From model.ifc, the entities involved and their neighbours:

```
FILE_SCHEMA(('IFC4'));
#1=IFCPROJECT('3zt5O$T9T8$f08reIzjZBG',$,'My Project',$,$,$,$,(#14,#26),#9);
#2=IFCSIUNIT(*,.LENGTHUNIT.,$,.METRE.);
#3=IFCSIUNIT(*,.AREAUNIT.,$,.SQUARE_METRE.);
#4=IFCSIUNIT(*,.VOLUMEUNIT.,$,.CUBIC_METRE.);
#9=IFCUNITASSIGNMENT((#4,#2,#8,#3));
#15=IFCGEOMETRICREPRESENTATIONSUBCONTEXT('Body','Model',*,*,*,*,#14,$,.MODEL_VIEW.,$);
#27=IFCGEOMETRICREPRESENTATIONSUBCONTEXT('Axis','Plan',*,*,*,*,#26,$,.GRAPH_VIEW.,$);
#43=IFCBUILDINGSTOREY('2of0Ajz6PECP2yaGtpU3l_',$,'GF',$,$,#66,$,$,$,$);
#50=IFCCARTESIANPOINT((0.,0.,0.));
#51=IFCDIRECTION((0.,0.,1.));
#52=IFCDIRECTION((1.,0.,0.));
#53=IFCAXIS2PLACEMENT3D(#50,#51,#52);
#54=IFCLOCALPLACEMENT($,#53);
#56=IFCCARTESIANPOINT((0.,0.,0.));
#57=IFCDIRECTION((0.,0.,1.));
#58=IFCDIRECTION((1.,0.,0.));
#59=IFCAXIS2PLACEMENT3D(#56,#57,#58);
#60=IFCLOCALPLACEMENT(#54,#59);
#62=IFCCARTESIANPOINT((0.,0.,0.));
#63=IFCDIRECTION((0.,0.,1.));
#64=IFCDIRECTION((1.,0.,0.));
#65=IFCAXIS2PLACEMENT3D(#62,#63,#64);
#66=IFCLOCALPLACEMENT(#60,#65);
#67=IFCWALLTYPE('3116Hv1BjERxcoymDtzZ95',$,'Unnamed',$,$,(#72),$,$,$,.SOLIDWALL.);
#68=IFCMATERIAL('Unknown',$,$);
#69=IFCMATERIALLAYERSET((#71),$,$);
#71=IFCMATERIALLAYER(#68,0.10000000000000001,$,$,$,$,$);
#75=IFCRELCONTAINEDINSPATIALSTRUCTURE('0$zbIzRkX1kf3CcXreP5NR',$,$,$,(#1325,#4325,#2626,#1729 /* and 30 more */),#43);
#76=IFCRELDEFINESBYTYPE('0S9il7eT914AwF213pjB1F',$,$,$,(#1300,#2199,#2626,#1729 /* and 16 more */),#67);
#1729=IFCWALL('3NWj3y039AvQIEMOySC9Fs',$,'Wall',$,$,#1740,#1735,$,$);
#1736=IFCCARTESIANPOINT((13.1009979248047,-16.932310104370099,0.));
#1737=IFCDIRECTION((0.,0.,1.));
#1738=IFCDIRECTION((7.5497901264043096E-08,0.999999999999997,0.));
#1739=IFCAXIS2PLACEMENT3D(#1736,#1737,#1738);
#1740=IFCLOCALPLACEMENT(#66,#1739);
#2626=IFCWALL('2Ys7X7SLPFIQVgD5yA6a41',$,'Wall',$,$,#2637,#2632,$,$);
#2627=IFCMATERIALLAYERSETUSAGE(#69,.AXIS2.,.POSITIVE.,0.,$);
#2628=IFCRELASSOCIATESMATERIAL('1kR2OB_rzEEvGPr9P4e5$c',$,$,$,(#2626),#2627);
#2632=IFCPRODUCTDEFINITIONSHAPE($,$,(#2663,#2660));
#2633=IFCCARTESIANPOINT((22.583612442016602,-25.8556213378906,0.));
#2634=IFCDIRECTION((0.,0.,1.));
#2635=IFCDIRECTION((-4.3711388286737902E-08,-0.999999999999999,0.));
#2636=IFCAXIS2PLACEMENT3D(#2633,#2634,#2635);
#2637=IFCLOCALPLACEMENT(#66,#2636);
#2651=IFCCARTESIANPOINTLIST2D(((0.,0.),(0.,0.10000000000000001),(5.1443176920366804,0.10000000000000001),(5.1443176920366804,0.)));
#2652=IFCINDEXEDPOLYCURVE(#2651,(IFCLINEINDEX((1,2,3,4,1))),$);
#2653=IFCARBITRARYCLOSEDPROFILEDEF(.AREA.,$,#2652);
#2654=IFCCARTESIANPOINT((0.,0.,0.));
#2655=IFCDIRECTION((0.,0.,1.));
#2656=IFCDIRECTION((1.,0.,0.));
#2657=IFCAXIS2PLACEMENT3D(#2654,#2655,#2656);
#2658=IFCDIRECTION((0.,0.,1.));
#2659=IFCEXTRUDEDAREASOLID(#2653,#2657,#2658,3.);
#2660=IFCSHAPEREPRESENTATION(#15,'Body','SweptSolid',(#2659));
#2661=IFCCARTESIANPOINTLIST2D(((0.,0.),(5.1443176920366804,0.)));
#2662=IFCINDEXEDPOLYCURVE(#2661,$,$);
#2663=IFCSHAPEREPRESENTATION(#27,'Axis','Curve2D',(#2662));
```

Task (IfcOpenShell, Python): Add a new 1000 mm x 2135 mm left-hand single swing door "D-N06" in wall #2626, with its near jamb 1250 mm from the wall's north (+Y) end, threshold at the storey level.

```python
import numpy as np
import ifcopenshell
import ifcopenshell.api.feature
import ifcopenshell.api.geometry
import ifcopenshell.api.root
import ifcopenshell.api.spatial
import ifcopenshell.geom
import ifcopenshell.util.element
import ifcopenshell.util.placement
import ifcopenshell.util.representation
import ifcopenshell.util.shape
import ifcopenshell.util.unit

model = ifcopenshell.open("model.ifc")
unit_scale = ifcopenshell.util.unit.calculate_unit_scale(model)
settings = ifcopenshell.geom.settings()


def volume(element):
    """Net volume in cubic metres, openings subtracted."""
    shape = ifcopenshell.geom.create_shape(settings, element)
    return ifcopenshell.util.shape.get_volume(shape.geometry)


wall = model.by_guid("2Ys7X7SLPFIQVgD5yA6a41")
storey = ifcopenshell.util.element.get_container(wall, ifc_class="IfcBuildingStorey")
context = ifcopenshell.util.representation.get_context(model, "Model", "Body", "MODEL_VIEW")
before = volume(wall)

width, height, from_end, sill = 1, 2.135, 1.25, 0.0  # metres

# The wall runs along its own X axis, and the end named is its -X end.
wall_shape = ifcopenshell.geom.create_shape(settings, wall)
x, y, z = ifcopenshell.util.shape.get_vertices(wall_shape.geometry).T
start = x.min() + from_end
face, thickness = float(y.min()), float(y.max() - y.min())
wall_matrix = ifcopenshell.util.placement.get_local_placement(wall.ObjectPlacement)
level = ifcopenshell.util.placement.get_local_placement(storey.ObjectPlacement)[2, 3]


def in_wall(x, y):
    """Placement at x, y metres in the wall's axes, at sill height."""
    matrix = wall_matrix.copy()
    matrix[:, 3] = wall_matrix @ np.array([x / unit_scale, y / unit_scale, 0.0, 1.0])
    matrix[2, 3] = level + sill / unit_scale
    return matrix


# Opening: a box that overshoots both wall faces by 50 mm.
opening = ifcopenshell.api.root.create_entity(model, ifc_class="IfcOpeningElement", predefined_type="OPENING")
box = ifcopenshell.api.geometry.add_wall_representation(
    model, context=context, length=width, height=height, thickness=thickness + 0.1
)
ifcopenshell.api.geometry.assign_representation(model, product=opening, representation=box)
ifcopenshell.api.geometry.edit_object_placement(model, product=opening, matrix=in_wall(start, face - 0.05), is_si=False)
ifcopenshell.api.feature.add_feature(model, feature=opening, element=wall)

door = ifcopenshell.api.root.create_entity(model, ifc_class="IfcDoor", name="D-N06", predefined_type="DOOR")
door.OverallWidth, door.OverallHeight = width / unit_scale, height / unit_scale
door.OperationType = "SINGLE_SWING_LEFT"
body = ifcopenshell.api.geometry.add_door_representation(
    model,
    context=context,
    overall_width=door.OverallWidth,
    overall_height=door.OverallHeight,
    operation_type="SINGLE_SWING_LEFT",
    lining_properties={"LiningDepth": thickness / unit_scale, "ThresholdDepth": thickness / unit_scale},
)
ifcopenshell.api.geometry.assign_representation(model, product=door, representation=body)
ifcopenshell.api.spatial.assign_container(model, products=[door], relating_structure=storey)
ifcopenshell.api.feature.add_filling(model, opening=opening, element=door)

# The lining spans the wall, so the door starts at the wall face.
ifcopenshell.api.geometry.edit_object_placement(model, product=door, matrix=in_wall(start, face), is_si=False)

after = volume(wall)

print(f"wall volume {before:.3f} -> {after:.3f} m3")

model.write("model_rev.ifc")
```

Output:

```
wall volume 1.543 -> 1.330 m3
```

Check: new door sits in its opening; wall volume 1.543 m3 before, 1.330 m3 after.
